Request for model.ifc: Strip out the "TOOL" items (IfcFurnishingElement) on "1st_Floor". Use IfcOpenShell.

First a look at what the model holds.

```python
import ifcopenshell
import ifcopenshell.util.element

model = ifcopenshell.open("model.ifc")
print(model.schema)
storey = next(s for s in model.by_type("IfcBuildingStorey") if s.Name == "1st_Floor")
furniture = [e for e in ifcopenshell.util.element.get_decomposition(storey) if e.is_a("IfcFurnishingElement")]
seen = {}
for e in furniture:
    element_type = ifcopenshell.util.element.get_type(e)
    name = element_type.Name if element_type not in (None, e) else None
    seen[name] = seen.get(name, 0) + 1
for name, count in sorted(seen.items(), key=str):
    print(count, "x", name)
```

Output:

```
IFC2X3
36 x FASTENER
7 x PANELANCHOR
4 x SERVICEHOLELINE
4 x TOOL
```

```python
import ifcopenshell
import ifcopenshell.api.root
import ifcopenshell.util.element

model = ifcopenshell.open("model.ifc")

storey = next(s for s in model.by_type("IfcBuildingStorey") if s.Name == "1st_Floor")
furniture = [e for e in ifcopenshell.util.element.get_decomposition(storey) if e.is_a("IfcFurnishingElement")]
targets = [e for e in furniture if (t := ifcopenshell.util.element.get_type(e)) not in (None, e) and t.Name == "TOOL"]

for e in targets:
    ifcopenshell.api.root.remove_product(model, product=e)
print(len(targets), "removed")

model.write("model_v2.ifc")
```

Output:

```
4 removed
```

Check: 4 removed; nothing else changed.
